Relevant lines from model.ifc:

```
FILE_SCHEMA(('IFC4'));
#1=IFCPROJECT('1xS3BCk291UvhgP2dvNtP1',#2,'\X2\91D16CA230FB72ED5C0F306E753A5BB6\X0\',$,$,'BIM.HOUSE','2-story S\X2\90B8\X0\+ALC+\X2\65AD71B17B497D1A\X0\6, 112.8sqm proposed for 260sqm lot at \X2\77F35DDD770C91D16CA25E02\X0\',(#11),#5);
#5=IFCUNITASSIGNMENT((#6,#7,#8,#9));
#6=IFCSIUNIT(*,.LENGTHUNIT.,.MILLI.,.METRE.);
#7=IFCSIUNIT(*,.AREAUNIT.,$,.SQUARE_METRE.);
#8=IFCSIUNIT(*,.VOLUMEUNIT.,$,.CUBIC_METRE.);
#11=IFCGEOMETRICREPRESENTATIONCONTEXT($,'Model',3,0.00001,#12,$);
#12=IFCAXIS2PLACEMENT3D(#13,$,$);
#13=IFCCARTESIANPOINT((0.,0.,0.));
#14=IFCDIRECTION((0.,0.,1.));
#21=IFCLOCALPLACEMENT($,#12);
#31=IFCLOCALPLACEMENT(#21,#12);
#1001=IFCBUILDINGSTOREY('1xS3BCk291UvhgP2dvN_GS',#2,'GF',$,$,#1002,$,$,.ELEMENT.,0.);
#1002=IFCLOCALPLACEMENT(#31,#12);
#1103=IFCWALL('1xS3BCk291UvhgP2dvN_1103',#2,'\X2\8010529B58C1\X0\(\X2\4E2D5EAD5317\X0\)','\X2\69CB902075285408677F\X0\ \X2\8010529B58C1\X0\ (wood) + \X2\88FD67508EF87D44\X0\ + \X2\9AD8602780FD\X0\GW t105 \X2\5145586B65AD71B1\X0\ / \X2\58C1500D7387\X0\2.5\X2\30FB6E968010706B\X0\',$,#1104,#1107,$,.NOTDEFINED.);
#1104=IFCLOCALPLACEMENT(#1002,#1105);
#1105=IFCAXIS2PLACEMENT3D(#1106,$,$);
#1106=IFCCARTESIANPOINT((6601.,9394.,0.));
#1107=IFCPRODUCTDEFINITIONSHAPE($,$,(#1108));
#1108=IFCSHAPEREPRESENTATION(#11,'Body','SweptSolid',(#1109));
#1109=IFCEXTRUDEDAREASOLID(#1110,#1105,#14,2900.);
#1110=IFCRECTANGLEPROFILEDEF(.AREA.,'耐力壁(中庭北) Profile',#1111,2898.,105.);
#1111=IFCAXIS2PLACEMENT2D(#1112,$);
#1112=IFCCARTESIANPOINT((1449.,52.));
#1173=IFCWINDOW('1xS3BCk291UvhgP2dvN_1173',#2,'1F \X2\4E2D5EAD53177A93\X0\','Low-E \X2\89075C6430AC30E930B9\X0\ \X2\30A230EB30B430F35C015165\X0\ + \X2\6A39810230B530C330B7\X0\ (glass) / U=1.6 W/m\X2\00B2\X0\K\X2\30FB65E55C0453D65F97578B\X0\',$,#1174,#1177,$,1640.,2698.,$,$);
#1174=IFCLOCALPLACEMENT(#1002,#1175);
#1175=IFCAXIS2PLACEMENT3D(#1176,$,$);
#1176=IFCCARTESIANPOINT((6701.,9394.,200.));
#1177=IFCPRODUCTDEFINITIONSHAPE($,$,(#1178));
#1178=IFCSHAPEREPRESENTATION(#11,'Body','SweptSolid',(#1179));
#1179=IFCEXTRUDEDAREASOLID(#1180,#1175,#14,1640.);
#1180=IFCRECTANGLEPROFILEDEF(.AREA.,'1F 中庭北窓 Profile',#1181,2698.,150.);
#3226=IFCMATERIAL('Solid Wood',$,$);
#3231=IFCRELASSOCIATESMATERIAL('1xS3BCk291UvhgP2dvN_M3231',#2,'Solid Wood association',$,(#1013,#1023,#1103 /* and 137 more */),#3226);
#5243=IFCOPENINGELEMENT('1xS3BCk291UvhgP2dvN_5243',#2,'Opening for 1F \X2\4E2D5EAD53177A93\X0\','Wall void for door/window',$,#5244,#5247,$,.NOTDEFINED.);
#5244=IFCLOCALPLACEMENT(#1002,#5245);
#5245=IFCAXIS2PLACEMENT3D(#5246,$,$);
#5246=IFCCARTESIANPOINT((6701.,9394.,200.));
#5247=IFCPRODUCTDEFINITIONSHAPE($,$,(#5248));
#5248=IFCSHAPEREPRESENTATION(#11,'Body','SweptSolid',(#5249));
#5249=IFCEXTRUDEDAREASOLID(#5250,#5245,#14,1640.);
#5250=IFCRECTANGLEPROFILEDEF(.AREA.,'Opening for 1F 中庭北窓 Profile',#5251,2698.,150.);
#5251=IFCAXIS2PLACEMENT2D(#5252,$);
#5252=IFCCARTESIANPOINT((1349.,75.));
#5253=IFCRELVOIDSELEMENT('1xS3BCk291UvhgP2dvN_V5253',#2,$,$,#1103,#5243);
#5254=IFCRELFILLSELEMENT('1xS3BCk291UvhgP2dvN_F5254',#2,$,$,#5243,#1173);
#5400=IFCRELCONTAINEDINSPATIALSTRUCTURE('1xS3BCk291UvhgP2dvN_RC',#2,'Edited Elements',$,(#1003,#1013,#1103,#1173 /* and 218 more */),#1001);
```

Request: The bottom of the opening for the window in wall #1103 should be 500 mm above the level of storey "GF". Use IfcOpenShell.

```python
import numpy as np
import ifcopenshell
import ifcopenshell.api.geometry
import ifcopenshell.geom
import ifcopenshell.util.element
import ifcopenshell.util.placement
import ifcopenshell.util.shape
import ifcopenshell.util.unit

model = ifcopenshell.open("model.ifc")
unit_scale = ifcopenshell.util.unit.calculate_unit_scale(model)

window = model.by_guid("1xS3BCk291UvhgP2dvN_1173")
opening = window.FillsVoids[0].RelatingOpeningElement
storey = ifcopenshell.util.element.get_container(window, ifc_class="IfcBuildingStorey")
level = ifcopenshell.util.placement.get_local_placement(storey.ObjectPlacement)[2, 3]

# The opening's origin need not be at the sill, so measure its lowest point.
shape = ifcopenshell.geom.create_shape(ifcopenshell.geom.settings(), opening)
bottom = ifcopenshell.util.shape.get_shape_bottom_elevation(shape, shape.geometry) / unit_scale
dz = level + 500.0 - bottom

shift = np.array([0.0, 0.0, dz])
# The window is not placed relative to its opening, so move both.
for product in (opening, window):
    matrix = ifcopenshell.util.placement.get_local_placement(product.ObjectPlacement)
    matrix[:3, 3] += shift
    ifcopenshell.api.geometry.edit_object_placement(model, product=product, matrix=matrix, is_si=False)

print(f"moved by {dz * unit_scale:+.3f} m")

model.write("model_updated.ifc")
```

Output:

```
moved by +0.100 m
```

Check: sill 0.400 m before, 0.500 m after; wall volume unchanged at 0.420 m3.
